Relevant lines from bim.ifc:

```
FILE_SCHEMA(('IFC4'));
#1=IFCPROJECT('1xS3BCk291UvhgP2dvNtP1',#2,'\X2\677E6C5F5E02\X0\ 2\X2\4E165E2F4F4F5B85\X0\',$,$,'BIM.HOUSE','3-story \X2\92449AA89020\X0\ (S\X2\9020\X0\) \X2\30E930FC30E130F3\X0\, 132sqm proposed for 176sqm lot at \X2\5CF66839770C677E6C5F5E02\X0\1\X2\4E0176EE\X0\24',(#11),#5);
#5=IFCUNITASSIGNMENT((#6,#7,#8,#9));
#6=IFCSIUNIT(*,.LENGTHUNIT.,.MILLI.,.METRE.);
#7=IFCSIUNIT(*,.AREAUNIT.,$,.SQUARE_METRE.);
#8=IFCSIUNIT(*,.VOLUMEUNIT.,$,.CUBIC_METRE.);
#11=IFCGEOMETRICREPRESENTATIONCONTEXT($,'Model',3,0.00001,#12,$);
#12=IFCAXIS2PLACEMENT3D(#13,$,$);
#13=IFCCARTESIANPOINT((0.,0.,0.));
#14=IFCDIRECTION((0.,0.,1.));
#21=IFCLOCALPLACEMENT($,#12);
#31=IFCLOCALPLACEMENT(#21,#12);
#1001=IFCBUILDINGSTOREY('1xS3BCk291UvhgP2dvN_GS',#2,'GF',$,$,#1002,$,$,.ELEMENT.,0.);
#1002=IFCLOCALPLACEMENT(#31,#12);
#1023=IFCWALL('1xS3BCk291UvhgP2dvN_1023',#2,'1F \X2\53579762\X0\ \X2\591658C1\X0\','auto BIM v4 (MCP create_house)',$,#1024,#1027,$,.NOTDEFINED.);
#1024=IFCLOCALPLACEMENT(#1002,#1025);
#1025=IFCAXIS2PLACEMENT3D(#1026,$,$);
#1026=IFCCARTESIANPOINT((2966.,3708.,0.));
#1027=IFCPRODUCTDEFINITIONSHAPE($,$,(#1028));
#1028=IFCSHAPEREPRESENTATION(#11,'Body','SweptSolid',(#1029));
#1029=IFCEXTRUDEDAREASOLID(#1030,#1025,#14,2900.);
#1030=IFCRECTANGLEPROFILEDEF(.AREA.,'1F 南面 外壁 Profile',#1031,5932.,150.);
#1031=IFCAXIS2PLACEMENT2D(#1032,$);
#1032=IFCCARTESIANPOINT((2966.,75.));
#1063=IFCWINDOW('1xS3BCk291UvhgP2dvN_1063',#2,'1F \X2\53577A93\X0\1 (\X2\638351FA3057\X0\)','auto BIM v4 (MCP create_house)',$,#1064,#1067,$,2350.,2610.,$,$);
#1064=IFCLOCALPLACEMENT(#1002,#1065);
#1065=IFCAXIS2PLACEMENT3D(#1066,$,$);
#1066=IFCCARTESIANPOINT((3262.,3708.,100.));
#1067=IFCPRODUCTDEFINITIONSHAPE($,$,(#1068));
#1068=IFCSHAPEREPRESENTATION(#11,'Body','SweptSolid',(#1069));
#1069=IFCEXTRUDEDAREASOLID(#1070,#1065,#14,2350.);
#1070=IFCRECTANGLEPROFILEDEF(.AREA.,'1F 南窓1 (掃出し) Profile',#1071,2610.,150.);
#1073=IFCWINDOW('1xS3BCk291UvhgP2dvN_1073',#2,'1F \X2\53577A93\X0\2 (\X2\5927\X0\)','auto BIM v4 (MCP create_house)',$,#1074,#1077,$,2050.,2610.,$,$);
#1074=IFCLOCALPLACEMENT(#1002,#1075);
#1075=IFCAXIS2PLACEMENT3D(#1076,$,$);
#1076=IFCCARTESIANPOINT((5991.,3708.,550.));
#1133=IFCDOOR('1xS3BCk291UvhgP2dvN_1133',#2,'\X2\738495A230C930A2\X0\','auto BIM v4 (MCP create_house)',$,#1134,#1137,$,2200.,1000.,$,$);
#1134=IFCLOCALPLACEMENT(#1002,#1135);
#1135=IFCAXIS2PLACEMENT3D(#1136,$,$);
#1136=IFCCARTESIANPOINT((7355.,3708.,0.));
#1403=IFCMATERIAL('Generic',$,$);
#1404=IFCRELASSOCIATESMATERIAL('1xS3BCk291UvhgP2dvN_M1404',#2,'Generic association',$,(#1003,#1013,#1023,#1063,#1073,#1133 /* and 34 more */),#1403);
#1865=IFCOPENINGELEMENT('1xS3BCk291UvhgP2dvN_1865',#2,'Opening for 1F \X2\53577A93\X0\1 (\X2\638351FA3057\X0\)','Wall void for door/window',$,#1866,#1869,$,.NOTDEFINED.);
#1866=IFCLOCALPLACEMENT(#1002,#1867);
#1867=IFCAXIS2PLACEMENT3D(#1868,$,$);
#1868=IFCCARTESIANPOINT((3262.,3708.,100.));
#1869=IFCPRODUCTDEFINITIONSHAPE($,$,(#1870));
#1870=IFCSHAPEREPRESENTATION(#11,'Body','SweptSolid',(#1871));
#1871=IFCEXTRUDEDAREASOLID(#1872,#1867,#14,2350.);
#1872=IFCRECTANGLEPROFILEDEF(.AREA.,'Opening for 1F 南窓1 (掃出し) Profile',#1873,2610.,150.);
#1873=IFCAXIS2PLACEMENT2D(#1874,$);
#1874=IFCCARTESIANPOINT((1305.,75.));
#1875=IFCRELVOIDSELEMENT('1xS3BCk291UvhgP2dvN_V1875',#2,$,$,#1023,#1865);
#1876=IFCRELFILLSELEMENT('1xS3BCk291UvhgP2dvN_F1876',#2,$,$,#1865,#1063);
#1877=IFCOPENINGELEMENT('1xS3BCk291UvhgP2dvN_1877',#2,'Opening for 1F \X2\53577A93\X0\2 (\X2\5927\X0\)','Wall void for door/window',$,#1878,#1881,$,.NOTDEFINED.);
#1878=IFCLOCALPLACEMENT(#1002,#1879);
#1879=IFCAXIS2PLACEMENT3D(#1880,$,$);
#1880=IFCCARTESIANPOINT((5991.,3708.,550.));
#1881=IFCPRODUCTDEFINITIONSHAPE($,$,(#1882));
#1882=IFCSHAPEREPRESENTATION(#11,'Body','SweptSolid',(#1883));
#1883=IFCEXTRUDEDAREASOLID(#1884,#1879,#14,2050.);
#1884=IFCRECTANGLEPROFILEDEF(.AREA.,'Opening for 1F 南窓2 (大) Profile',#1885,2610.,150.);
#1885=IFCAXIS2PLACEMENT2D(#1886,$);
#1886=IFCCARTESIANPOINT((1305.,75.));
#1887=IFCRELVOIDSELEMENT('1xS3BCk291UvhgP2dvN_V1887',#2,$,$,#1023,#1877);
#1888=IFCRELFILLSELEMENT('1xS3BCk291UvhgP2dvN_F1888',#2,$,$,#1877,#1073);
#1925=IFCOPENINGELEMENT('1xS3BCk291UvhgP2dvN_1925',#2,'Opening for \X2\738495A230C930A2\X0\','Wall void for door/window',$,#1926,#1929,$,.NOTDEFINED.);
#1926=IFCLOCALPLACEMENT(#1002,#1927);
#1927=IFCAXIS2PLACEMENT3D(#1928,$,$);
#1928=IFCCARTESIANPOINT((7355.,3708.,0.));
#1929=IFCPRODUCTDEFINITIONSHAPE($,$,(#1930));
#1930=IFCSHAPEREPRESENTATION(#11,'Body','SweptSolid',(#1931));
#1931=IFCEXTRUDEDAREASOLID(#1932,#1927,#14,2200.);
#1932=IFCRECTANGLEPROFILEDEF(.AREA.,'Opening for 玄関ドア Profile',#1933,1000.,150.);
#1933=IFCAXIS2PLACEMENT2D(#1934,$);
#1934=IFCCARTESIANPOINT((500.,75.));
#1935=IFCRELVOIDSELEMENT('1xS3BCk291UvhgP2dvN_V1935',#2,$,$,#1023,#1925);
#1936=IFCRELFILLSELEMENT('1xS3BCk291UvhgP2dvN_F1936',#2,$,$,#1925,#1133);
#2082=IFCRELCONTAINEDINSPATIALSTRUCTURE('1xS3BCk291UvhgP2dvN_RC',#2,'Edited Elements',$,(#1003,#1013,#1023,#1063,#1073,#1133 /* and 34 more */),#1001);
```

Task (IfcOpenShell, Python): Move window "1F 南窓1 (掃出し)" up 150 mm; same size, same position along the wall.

```python
import numpy as np
import ifcopenshell
import ifcopenshell.api.geometry
import ifcopenshell.util.placement
import ifcopenshell.util.unit

model = ifcopenshell.open("bim.ifc")
unit_scale = ifcopenshell.util.unit.calculate_unit_scale(model)

window = model.by_guid("1xS3BCk291UvhgP2dvN_1063")
opening = window.FillsVoids[0].RelatingOpeningElement
dz = 150.0

shift = np.array([0.0, 0.0, dz])
# The window is not placed relative to its opening, so move both.
for product in (opening, window):
    matrix = ifcopenshell.util.placement.get_local_placement(product.ObjectPlacement)
    matrix[:3, 3] += shift
    ifcopenshell.api.geometry.edit_object_placement(model, product=product, matrix=matrix, is_si=False)

print(f"moved by {dz * unit_scale:+.3f} m")

model.write("bim_rev.ifc")
```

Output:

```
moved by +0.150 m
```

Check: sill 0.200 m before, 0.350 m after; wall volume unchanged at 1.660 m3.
